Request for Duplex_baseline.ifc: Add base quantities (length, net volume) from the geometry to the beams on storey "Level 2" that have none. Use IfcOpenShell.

First a look at what the model holds.

```python
import ifcopenshell
import ifcopenshell.util.element
import ifcopenshell.util.unit

model = ifcopenshell.open("Duplex_baseline.ifc")
print(model.schema)
for unit_type in ("LENGTHUNIT", "AREAUNIT", "VOLUMEUNIT"):
    print(unit_type, ifcopenshell.util.unit.calculate_unit_scale(model, unit_type))
storey = next(s for s in model.by_type("IfcBuildingStorey") if s.Name == "Level 2")
beams = [e for e in ifcopenshell.util.element.get_decomposition(storey) if e.is_a("IfcBeam")]
for e in sorted(beams, key=lambda e: e.id()):
    print(e.id(), e.is_a(), e.Name, list(ifcopenshell.util.element.get_psets(e, qtos_only=True)), sep=" | ")
```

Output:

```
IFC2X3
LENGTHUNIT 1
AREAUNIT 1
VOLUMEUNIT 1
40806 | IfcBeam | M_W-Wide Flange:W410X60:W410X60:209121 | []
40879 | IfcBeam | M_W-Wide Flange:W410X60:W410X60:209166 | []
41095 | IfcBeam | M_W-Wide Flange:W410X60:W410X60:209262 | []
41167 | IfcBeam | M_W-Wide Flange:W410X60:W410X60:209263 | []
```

```python
import ifcopenshell
import ifcopenshell.api.pset
import ifcopenshell.geom
import ifcopenshell.util.element
import ifcopenshell.util.shape
import ifcopenshell.util.unit

model = ifcopenshell.open("Duplex_baseline.ifc")
unit_scale = ifcopenshell.util.unit.calculate_unit_scale(model)
volume_scale = ifcopenshell.util.unit.calculate_unit_scale(model, "VOLUMEUNIT")
settings = ifcopenshell.geom.settings()

storey = next(s for s in model.by_type("IfcBuildingStorey") if s.Name == "Level 2")
beams = [e for e in ifcopenshell.util.element.get_decomposition(storey) if e.is_a("IfcBeam")]

for e in sorted(beams, key=lambda e: e.id()):
    if ifcopenshell.util.element.get_psets(e, qtos_only=True, should_inherit=False):
        continue
    # Geometry comes back in metres, in the element's own axes.
    shape = ifcopenshell.geom.create_shape(settings, e)
    values = {
        "Length": ifcopenshell.util.shape.get_max_xyz(shape.geometry) / unit_scale,
        "NetVolume": ifcopenshell.util.shape.get_volume(shape.geometry) / volume_scale,
    }
    qto = ifcopenshell.api.pset.add_qto(model, product=e, name="BaseQuantities")
    ifcopenshell.api.pset.edit_qto(model, qto=qto, properties=values)
    print(e.id(), {k: round(v, 3) for k, v in values.items()})

model.write("Duplex_baseline-out.ifc")
```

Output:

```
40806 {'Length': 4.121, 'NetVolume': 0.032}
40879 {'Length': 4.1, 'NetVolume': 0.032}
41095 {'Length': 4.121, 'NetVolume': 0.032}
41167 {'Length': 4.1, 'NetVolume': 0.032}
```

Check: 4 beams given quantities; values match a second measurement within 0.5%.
